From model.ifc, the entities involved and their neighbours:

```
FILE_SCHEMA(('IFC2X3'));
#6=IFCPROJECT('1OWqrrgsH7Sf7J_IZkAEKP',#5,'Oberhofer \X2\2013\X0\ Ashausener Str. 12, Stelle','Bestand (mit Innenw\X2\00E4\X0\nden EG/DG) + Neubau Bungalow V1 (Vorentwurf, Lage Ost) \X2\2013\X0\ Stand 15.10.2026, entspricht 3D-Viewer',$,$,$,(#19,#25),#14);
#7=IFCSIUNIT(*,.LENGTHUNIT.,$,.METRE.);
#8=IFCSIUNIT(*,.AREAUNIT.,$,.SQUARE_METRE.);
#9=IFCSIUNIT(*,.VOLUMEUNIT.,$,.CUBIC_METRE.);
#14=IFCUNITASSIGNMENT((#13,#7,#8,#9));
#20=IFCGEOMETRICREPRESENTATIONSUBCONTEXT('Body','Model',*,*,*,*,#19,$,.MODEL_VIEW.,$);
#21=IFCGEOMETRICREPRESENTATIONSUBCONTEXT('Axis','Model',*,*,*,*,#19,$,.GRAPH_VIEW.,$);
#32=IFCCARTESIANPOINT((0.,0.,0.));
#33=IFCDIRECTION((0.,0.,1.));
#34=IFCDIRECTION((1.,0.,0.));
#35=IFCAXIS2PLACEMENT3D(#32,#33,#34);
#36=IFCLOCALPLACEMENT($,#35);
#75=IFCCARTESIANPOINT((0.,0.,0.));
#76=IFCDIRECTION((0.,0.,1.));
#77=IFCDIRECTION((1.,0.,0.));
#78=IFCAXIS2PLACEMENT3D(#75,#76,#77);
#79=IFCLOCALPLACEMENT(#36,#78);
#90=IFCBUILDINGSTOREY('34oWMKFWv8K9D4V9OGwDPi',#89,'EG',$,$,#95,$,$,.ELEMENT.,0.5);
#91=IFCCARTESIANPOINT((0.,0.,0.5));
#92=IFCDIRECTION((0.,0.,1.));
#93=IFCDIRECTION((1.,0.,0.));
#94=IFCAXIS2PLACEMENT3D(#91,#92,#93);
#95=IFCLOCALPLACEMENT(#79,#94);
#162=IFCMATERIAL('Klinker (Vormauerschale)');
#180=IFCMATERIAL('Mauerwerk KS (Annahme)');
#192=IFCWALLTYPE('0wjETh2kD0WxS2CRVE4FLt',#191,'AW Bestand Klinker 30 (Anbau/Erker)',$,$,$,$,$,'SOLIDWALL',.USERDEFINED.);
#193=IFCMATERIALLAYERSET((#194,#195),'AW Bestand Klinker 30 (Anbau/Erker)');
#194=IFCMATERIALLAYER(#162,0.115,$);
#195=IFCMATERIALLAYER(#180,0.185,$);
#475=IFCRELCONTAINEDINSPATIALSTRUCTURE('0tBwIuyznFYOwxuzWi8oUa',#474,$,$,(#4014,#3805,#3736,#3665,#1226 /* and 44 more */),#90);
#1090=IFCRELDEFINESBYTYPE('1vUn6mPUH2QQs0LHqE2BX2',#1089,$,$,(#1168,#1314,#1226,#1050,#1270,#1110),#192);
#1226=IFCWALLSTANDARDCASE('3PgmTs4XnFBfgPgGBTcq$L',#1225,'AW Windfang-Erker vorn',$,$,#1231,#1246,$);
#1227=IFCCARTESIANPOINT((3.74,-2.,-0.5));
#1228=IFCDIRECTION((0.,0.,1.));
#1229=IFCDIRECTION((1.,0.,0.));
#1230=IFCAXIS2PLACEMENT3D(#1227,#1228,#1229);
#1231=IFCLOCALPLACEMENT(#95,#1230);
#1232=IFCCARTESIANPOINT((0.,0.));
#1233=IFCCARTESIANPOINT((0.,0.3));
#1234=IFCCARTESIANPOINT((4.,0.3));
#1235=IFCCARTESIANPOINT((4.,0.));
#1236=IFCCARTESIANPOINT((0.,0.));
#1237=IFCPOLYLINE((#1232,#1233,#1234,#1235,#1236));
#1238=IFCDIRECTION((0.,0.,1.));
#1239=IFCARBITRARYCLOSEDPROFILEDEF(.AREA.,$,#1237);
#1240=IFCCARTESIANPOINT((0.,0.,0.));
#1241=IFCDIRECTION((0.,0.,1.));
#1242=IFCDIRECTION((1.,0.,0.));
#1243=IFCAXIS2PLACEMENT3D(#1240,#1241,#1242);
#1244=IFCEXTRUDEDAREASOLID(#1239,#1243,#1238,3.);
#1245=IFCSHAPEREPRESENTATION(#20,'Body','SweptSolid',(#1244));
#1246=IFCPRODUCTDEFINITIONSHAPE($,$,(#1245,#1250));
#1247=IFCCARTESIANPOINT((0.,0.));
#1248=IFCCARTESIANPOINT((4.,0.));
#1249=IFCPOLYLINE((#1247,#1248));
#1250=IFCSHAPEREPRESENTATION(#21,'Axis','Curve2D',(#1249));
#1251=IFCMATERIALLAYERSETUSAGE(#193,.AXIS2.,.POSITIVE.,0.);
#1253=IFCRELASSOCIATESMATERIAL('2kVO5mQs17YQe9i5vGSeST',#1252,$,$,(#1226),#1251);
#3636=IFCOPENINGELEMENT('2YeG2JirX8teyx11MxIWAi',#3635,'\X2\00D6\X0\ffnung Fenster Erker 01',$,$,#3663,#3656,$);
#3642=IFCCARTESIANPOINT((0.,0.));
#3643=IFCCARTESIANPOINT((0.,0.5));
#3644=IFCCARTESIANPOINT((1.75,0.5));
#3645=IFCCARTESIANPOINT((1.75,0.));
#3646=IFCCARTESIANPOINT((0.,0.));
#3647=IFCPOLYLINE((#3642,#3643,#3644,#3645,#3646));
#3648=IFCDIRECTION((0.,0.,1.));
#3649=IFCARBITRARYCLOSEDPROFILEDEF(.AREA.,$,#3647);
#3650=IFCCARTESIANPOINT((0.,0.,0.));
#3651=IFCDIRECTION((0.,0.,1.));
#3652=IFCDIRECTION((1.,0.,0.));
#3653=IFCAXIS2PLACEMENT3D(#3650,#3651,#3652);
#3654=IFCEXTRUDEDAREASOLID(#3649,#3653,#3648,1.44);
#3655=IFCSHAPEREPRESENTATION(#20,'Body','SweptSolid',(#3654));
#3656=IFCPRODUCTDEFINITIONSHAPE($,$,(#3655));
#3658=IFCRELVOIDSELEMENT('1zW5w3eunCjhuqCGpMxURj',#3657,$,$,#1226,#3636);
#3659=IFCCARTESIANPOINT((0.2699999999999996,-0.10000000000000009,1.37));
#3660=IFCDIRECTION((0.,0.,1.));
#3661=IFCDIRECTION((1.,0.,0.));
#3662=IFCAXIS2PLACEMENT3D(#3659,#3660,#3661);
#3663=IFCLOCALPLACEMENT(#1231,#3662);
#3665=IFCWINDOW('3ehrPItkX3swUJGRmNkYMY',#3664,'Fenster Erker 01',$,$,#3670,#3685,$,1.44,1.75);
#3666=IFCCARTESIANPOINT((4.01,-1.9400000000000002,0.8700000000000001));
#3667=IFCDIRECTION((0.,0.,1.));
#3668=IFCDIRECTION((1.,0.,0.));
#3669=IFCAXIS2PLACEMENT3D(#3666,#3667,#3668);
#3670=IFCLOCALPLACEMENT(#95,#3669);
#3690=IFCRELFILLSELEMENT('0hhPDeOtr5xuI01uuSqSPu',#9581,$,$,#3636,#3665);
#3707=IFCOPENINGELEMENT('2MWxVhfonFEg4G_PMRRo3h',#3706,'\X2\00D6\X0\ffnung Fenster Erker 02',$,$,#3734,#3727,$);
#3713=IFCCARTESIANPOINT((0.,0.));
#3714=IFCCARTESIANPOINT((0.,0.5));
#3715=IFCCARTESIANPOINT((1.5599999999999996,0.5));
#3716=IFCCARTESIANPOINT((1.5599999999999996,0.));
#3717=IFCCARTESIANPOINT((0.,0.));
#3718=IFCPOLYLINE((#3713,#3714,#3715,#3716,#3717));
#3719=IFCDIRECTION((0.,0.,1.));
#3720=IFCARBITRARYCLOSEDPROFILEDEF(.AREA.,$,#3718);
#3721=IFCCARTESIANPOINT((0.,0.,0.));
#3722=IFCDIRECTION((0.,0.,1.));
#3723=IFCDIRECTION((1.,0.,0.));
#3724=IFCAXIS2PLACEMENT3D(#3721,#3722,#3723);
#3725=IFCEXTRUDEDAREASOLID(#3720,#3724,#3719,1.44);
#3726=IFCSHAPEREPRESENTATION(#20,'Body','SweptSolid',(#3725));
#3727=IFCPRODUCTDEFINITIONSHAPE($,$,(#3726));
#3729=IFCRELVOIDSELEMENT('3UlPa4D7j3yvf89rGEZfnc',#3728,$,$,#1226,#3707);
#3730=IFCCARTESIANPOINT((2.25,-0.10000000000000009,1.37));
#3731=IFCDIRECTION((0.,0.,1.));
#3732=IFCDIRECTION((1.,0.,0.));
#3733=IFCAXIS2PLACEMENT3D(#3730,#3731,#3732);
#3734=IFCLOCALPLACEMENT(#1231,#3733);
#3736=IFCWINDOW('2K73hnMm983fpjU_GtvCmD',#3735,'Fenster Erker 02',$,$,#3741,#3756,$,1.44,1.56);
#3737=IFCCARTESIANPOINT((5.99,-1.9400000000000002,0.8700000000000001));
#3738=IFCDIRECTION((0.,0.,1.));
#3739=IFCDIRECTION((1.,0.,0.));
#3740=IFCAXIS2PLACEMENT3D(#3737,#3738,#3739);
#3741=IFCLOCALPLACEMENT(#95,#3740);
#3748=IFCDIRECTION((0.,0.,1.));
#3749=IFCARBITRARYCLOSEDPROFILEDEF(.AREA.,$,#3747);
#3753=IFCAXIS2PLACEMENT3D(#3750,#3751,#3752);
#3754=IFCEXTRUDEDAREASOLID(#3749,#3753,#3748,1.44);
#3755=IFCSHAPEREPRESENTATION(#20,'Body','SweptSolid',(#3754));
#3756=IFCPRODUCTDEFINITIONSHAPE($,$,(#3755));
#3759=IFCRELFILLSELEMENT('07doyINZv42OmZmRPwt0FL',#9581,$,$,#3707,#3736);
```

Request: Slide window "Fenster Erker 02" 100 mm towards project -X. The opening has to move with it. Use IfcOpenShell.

```python
import ifcopenshell
import ifcopenshell.api.geometry
import ifcopenshell.util.placement
import ifcopenshell.util.unit

model = ifcopenshell.open("model.ifc")
unit_scale = ifcopenshell.util.unit.calculate_unit_scale(model)

window = model.by_guid("2K73hnMm983fpjU_GtvCmD")
opening = window.FillsVoids[0].RelatingOpeningElement
wall = opening.VoidsElements[0].RelatingBuildingElement

wall_matrix = ifcopenshell.util.placement.get_local_placement(wall.ObjectPlacement)
shift = wall_matrix[:3, 0] * -0.1 / unit_scale
before = ifcopenshell.util.placement.get_local_placement(window.ObjectPlacement)[:3, 3].copy()

# The window is not placed relative to its opening, so move both.
for product in (opening, window):
    matrix = ifcopenshell.util.placement.get_local_placement(product.ObjectPlacement)
    matrix[:3, 3] += shift
    ifcopenshell.api.geometry.edit_object_placement(model, product=product, matrix=matrix, is_si=False)

after = ifcopenshell.util.placement.get_local_placement(window.ObjectPlacement)[:3, 3]
print("window moved by", (after - before).round(3) + 0.0)

model.write("model_rev.ifc")
```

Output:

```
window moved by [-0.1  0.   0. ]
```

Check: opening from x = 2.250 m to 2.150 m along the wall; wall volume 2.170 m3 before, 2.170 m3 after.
